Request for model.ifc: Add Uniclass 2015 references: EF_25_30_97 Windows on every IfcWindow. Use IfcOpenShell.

First a look at what the model holds.

```python
import ifcopenshell

model = ifcopenshell.open("model.ifc")
print(model.schema)
print("classifications:", [c.Name for c in model.by_type("IfcClassification")])
for ifc_class in ("IfcDoor", "IfcRoof", "IfcStair", "IfcWall", "IfcWindow"):
    print(ifc_class, len(model.by_type(ifc_class)))
```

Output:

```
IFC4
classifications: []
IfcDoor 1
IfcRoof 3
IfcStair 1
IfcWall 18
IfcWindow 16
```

```python
import ifcopenshell
import ifcopenshell.api.classification

model = ifcopenshell.open("model.ifc")

system = ifcopenshell.api.classification.add_classification(model, classification="Uniclass 2015")

codes = {
    "IfcWindow": ("EF_25_30_97", "Windows"),
}
for ifc_class, (code, name) in codes.items():
    products = model.by_type(ifc_class)
    ifcopenshell.api.classification.add_reference(
        model, products=products, classification=system, identification=code, name=name
    )
    print(code, len(products))

model.write("model_rev.ifc")
```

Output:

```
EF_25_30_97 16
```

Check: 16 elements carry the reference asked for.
